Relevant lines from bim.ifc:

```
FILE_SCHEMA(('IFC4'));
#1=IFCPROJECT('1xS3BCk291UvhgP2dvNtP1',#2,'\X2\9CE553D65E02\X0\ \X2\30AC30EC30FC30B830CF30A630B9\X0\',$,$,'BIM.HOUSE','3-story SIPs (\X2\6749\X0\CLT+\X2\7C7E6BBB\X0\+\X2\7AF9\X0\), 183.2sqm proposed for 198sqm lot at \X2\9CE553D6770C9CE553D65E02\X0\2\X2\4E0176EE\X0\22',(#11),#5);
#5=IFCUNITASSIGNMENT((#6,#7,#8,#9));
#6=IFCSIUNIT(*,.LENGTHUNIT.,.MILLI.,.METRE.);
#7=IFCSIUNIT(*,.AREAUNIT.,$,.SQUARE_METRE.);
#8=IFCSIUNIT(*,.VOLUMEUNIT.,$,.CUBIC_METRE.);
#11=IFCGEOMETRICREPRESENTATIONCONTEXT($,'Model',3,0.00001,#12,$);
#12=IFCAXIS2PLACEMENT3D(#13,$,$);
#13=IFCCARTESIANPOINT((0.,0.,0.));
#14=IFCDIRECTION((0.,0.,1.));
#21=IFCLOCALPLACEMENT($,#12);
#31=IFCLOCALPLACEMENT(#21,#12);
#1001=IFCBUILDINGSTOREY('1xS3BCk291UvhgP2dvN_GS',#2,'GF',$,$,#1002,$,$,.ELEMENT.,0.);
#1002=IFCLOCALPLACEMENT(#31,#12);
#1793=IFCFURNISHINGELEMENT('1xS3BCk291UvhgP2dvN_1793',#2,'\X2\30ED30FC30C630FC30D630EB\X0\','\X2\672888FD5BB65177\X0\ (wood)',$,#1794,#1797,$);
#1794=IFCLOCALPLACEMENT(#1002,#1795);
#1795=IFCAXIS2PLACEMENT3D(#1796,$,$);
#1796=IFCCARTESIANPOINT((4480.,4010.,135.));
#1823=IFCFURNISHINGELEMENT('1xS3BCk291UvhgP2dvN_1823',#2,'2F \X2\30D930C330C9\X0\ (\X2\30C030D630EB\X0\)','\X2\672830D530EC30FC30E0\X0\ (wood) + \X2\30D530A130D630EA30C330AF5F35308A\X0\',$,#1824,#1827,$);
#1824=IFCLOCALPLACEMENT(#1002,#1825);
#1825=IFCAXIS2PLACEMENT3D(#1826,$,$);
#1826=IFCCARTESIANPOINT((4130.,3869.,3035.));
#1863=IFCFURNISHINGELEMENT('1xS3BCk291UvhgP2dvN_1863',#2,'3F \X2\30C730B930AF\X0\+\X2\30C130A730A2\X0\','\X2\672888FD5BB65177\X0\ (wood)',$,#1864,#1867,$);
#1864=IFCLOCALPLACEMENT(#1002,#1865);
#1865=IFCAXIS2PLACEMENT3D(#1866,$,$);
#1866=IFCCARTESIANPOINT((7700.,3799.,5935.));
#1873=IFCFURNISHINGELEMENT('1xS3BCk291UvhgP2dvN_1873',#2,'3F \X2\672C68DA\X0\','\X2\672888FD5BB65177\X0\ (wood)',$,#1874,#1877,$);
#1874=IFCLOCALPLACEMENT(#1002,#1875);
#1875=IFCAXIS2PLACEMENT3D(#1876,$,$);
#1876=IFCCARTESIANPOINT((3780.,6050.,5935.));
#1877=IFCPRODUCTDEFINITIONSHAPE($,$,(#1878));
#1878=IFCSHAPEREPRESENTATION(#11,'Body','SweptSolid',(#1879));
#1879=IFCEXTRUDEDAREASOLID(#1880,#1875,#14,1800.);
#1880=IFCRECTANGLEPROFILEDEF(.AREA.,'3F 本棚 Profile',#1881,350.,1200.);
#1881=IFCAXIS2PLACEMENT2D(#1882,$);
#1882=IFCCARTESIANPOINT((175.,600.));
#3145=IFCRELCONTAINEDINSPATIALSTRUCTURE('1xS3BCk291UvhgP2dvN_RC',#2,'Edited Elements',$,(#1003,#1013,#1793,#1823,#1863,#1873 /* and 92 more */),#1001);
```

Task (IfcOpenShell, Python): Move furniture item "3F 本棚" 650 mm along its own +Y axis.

```python
import ifcopenshell
import ifcopenshell.api.geometry
import ifcopenshell.util.placement
import ifcopenshell.util.unit

model = ifcopenshell.open("bim.ifc")
unit_scale = ifcopenshell.util.unit.calculate_unit_scale(model)

item = model.by_guid("1xS3BCk291UvhgP2dvN_1873")
matrix = ifcopenshell.util.placement.get_local_placement(item.ObjectPlacement)
matrix[:3, 3] += matrix[:3, 1] * 0.65 / unit_scale
ifcopenshell.api.geometry.edit_object_placement(model, product=item, matrix=matrix, is_si=False)

print(ifcopenshell.util.placement.get_local_placement(item.ObjectPlacement).round(3) + 0.0)

model.write("bim_rev.ifc")
```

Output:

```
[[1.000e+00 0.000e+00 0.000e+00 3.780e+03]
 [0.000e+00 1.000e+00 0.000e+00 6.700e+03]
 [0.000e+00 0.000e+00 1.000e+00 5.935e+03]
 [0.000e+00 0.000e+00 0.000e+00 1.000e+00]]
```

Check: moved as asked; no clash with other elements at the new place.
